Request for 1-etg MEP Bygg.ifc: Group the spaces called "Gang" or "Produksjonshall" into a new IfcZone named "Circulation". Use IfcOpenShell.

First a look at what the model holds.

```python
import ifcopenshell

model = ifcopenshell.open("1-etg MEP Bygg.ifc")
print(model.schema)
seen = {}
for space in model.by_type("IfcSpace"):
    seen[space.LongName] = seen.get(space.LongName, 0) + 1
for name, count in sorted(seen.items(), key=str):
    print(count, "x", name)
print("zones:", [z.Name for z in model.by_type("IfcZone")][:20])
```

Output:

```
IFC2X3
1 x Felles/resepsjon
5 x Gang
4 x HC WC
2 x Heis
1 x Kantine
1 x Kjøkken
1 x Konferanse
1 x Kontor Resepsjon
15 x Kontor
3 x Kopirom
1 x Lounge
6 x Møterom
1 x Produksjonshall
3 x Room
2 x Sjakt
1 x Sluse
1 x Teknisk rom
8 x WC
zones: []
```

```python
import ifcopenshell
import ifcopenshell.api.group
import ifcopenshell.api.root

model = ifcopenshell.open("1-etg MEP Bygg.ifc")

names = {"Gang", "Produksjonshall"}
spaces = [s for s in model.by_type("IfcSpace") if s.LongName in names]

zone = ifcopenshell.api.root.create_entity(model, ifc_class="IfcZone", name="Circulation")
ifcopenshell.api.group.assign_group(model, products=spaces, group=zone)
print(len(spaces), "spaces in", zone.Name)

model.write("1-etg MEP Bygg_updated.ifc")
```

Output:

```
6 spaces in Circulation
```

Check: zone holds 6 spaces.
